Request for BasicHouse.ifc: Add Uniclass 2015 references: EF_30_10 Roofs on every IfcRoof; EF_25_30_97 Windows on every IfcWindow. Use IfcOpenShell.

First a look at what the model holds.

```python
import ifcopenshell

model = ifcopenshell.open("BasicHouse.ifc")
print(model.schema)
print("classifications:", [c.Name for c in model.by_type("IfcClassification")])
for ifc_class in ("IfcDoor", "IfcRoof", "IfcStair", "IfcWall", "IfcWindow"):
    print(ifc_class, len(model.by_type(ifc_class)))
```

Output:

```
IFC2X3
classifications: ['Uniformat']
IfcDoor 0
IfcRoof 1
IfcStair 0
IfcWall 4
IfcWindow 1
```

```python
import ifcopenshell
import ifcopenshell.api.classification

model = ifcopenshell.open("BasicHouse.ifc")

# IFC2X3 requires Source and Edition and has no link from the project to the system.
system = model.create_entity("IfcClassification", Source="NBS", Edition="2015", Name="Uniclass 2015")

codes = {
    "IfcRoof": ("EF_30_10", "Roofs"),
    "IfcWindow": ("EF_25_30_97", "Windows"),
}
for ifc_class, (code, name) in codes.items():
    products = model.by_type(ifc_class)
    ifcopenshell.api.classification.add_reference(
        model, products=products, classification=system, identification=code, name=name
    )
    print(code, len(products))

model.write("BasicHouse_rev.ifc")
```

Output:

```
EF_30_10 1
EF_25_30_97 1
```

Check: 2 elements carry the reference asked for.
